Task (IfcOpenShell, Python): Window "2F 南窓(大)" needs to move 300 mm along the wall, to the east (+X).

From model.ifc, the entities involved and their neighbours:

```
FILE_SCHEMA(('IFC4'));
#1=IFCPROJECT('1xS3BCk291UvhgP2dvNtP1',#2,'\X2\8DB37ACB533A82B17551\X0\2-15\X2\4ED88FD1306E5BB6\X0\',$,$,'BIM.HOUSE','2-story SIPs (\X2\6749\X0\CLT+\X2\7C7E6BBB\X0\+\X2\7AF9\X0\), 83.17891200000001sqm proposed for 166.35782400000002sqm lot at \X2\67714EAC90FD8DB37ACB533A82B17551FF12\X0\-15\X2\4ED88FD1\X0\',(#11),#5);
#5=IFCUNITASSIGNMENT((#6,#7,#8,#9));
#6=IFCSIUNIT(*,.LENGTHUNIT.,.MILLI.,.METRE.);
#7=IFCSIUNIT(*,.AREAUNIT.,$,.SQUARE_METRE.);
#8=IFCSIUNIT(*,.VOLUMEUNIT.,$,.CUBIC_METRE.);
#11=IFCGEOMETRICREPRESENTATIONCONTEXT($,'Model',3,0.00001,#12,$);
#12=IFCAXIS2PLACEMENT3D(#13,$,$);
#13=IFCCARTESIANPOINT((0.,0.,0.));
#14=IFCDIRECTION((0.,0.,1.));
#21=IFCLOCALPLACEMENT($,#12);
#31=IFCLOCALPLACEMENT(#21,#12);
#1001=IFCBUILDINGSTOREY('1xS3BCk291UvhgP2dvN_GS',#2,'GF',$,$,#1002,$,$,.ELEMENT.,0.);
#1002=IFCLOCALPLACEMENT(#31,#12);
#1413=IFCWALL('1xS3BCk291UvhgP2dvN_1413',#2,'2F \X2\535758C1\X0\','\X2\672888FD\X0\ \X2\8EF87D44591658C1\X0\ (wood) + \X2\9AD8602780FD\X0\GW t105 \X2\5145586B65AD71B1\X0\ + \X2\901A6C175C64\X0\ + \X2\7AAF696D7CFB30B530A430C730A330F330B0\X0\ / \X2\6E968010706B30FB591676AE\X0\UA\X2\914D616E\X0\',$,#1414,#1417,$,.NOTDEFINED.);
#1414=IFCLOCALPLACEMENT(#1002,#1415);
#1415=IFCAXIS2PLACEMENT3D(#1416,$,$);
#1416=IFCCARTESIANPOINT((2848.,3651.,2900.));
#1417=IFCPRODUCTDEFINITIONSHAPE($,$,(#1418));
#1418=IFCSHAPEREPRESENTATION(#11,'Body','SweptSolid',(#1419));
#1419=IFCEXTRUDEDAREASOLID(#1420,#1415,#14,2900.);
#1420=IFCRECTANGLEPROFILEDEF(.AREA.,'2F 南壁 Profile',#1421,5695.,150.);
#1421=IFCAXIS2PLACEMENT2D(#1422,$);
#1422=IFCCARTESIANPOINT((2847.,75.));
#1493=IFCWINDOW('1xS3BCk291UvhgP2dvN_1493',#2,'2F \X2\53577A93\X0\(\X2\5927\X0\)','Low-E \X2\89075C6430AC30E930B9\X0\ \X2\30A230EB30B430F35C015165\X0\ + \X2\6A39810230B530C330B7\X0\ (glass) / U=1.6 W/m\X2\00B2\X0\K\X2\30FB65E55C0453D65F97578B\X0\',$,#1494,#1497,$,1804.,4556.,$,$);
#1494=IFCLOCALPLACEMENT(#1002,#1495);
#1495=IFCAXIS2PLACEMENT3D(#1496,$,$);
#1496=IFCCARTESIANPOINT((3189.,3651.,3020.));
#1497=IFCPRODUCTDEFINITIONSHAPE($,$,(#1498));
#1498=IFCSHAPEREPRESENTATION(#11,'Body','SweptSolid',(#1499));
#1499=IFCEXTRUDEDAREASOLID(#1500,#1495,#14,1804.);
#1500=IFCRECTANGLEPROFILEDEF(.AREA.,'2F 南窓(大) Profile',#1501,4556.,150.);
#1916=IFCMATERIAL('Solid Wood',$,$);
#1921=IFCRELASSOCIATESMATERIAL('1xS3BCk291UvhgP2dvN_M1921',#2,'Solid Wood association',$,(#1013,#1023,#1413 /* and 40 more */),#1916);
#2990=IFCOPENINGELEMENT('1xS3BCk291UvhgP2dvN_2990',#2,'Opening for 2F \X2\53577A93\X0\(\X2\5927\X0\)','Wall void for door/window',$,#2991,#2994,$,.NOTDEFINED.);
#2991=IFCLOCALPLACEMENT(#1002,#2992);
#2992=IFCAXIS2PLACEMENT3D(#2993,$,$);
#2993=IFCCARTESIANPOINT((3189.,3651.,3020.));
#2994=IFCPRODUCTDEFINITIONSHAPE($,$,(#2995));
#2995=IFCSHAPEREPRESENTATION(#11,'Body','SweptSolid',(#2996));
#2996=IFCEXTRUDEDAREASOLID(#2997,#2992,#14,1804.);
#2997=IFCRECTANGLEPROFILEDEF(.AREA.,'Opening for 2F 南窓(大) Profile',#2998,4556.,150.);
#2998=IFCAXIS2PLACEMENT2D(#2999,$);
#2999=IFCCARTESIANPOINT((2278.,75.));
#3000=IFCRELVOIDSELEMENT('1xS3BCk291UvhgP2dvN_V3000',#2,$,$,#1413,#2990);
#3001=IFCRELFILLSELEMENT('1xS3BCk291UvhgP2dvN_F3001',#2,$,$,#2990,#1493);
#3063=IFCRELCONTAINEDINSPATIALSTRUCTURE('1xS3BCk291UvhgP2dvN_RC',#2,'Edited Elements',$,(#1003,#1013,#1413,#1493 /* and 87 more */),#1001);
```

```python
import ifcopenshell
import ifcopenshell.api.geometry
import ifcopenshell.util.placement
import ifcopenshell.util.unit

model = ifcopenshell.open("model.ifc")
unit_scale = ifcopenshell.util.unit.calculate_unit_scale(model)

window = model.by_guid("1xS3BCk291UvhgP2dvN_1493")
opening = window.FillsVoids[0].RelatingOpeningElement
wall = opening.VoidsElements[0].RelatingBuildingElement

wall_matrix = ifcopenshell.util.placement.get_local_placement(wall.ObjectPlacement)
shift = wall_matrix[:3, 0] * 0.3 / unit_scale
before = ifcopenshell.util.placement.get_local_placement(window.ObjectPlacement)[:3, 3].copy()

# The window is not placed relative to its opening, so move both.
for product in (opening, window):
    matrix = ifcopenshell.util.placement.get_local_placement(product.ObjectPlacement)
    matrix[:3, 3] += shift
    ifcopenshell.api.geometry.edit_object_placement(model, product=product, matrix=matrix, is_si=False)

after = ifcopenshell.util.placement.get_local_placement(window.ObjectPlacement)[:3, 3]
print("window moved by", (after - before).round(3) + 0.0)

model.write("model_rev.ifc")
```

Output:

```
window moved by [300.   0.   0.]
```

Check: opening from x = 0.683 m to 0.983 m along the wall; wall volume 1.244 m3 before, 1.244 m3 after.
